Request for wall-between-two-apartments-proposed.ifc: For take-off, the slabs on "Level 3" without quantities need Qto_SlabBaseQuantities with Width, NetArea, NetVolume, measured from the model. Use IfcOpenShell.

First a look at what the model holds.

```python
import ifcopenshell
import ifcopenshell.util.element
import ifcopenshell.util.unit

model = ifcopenshell.open("wall-between-two-apartments-proposed.ifc")
print(model.schema)
for unit_type in ("LENGTHUNIT", "AREAUNIT", "VOLUMEUNIT"):
    print(unit_type, ifcopenshell.util.unit.calculate_unit_scale(model, unit_type))
storey = next(s for s in model.by_type("IfcBuildingStorey") if s.Name == "Level 3")
slabs = [e for e in ifcopenshell.util.element.get_decomposition(storey) if e.is_a("IfcSlab")]
for e in sorted(slabs, key=lambda e: e.id()):
    print(e.id(), e.is_a(), e.Name, list(ifcopenshell.util.element.get_psets(e, qtos_only=True)), sep=" | ")
```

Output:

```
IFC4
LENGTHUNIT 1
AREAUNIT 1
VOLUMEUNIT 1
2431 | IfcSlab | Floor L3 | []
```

```python
import ifcopenshell
import ifcopenshell.api.pset
import ifcopenshell.geom
import ifcopenshell.util.element
import ifcopenshell.util.shape
import ifcopenshell.util.unit

model = ifcopenshell.open("wall-between-two-apartments-proposed.ifc")
unit_scale = ifcopenshell.util.unit.calculate_unit_scale(model)
area_scale = ifcopenshell.util.unit.calculate_unit_scale(model, "AREAUNIT")
volume_scale = ifcopenshell.util.unit.calculate_unit_scale(model, "VOLUMEUNIT")
settings = ifcopenshell.geom.settings()

storey = next(s for s in model.by_type("IfcBuildingStorey") if s.Name == "Level 3")
slabs = [e for e in ifcopenshell.util.element.get_decomposition(storey) if e.is_a("IfcSlab")]

for e in sorted(slabs, key=lambda e: e.id()):
    if ifcopenshell.util.element.get_psets(e, qtos_only=True, should_inherit=False):
        continue
    # Geometry comes back in metres, in the element's own axes.
    shape = ifcopenshell.geom.create_shape(settings, e)
    values = {
        "Width": ifcopenshell.util.shape.get_z(shape.geometry) / unit_scale,
        "NetArea": ifcopenshell.util.shape.get_footprint_area(shape.geometry) / area_scale,
        "NetVolume": ifcopenshell.util.shape.get_volume(shape.geometry) / volume_scale,
    }
    qto = ifcopenshell.api.pset.add_qto(model, product=e, name="Qto_SlabBaseQuantities")
    ifcopenshell.api.pset.edit_qto(model, qto=qto, properties=values)
    print(e.id(), {k: round(v, 3) for k, v in values.items()})

model.write("wall-between-two-apartments-proposed-out.ifc")
```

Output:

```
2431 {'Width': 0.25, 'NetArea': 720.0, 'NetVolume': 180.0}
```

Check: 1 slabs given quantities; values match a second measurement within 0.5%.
